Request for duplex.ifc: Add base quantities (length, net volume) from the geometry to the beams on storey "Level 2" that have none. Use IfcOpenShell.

First a look at what the model holds.

```python
import ifcopenshell
import ifcopenshell.util.element
import ifcopenshell.util.unit

model = ifcopenshell.open("duplex.ifc")
print(model.schema)
for unit_type in ("LENGTHUNIT", "AREAUNIT", "VOLUMEUNIT"):
    print(unit_type, ifcopenshell.util.unit.calculate_unit_scale(model, unit_type))
storey = next(s for s in model.by_type("IfcBuildingStorey") if s.Name == "Level 2")
beams = [e for e in ifcopenshell.util.element.get_decomposition(storey) if e.is_a("IfcBeam")]
for e in sorted(beams, key=lambda e: e.id()):
    print(e.id(), e.is_a(), e.Name, list(ifcopenshell.util.element.get_psets(e, qtos_only=True)), sep=" | ")
```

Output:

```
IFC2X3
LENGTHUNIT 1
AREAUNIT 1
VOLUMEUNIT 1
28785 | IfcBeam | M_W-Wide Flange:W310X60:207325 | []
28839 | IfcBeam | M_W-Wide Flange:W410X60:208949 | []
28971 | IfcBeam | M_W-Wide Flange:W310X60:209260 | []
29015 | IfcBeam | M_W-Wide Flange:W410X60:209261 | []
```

```python
import ifcopenshell
import ifcopenshell.api.pset
import ifcopenshell.geom
import ifcopenshell.util.element
import ifcopenshell.util.shape
import ifcopenshell.util.unit

model = ifcopenshell.open("duplex.ifc")
unit_scale = ifcopenshell.util.unit.calculate_unit_scale(model)
volume_scale = ifcopenshell.util.unit.calculate_unit_scale(model, "VOLUMEUNIT")
settings = ifcopenshell.geom.settings()

storey = next(s for s in model.by_type("IfcBuildingStorey") if s.Name == "Level 2")
beams = [e for e in ifcopenshell.util.element.get_decomposition(storey) if e.is_a("IfcBeam")]

for e in sorted(beams, key=lambda e: e.id()):
    if ifcopenshell.util.element.get_psets(e, qtos_only=True, should_inherit=False):
        continue
    # Geometry comes back in metres, in the element's own axes.
    shape = ifcopenshell.geom.create_shape(settings, e)
    values = {
        "Length": ifcopenshell.util.shape.get_max_xyz(shape.geometry) / unit_scale,
        "NetVolume": ifcopenshell.util.shape.get_volume(shape.geometry) / volume_scale,
    }
    qto = ifcopenshell.api.pset.add_qto(model, product=e, name="BaseQuantities")
    ifcopenshell.api.pset.edit_qto(model, qto=qto, properties=values)
    print(e.id(), {k: round(v, 3) for k, v in values.items()})

model.write("duplex_v2.ifc")
```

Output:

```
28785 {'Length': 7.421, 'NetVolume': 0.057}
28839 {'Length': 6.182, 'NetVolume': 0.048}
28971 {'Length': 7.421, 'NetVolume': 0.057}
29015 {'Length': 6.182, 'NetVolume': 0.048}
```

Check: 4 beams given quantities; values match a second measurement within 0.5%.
